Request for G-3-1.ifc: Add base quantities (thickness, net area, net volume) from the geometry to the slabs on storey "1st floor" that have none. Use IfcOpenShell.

First a look at what the model holds.

```python
import ifcopenshell
import ifcopenshell.util.element
import ifcopenshell.util.unit

model = ifcopenshell.open("G-3-1.ifc")
print(model.schema)
for unit_type in ("LENGTHUNIT", "AREAUNIT", "VOLUMEUNIT"):
    print(unit_type, ifcopenshell.util.unit.calculate_unit_scale(model, unit_type))
storey = next(s for s in model.by_type("IfcBuildingStorey") if s.Name == "1st floor")
slabs = [e for e in ifcopenshell.util.element.get_decomposition(storey) if e.is_a("IfcSlab")]
for e in sorted(slabs, key=lambda e: e.id()):
    print(e.id(), e.is_a(), e.Name, list(ifcopenshell.util.element.get_psets(e, qtos_only=True)), sep=" | ")
```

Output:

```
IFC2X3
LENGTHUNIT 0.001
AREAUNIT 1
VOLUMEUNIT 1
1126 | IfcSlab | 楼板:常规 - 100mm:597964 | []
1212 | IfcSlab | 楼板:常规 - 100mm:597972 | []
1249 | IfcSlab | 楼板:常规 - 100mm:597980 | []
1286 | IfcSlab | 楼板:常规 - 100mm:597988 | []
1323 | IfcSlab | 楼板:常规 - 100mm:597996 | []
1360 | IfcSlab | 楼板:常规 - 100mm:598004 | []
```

```python
import ifcopenshell
import ifcopenshell.api.pset
import ifcopenshell.geom
import ifcopenshell.util.element
import ifcopenshell.util.shape
import ifcopenshell.util.unit

model = ifcopenshell.open("G-3-1.ifc")
unit_scale = ifcopenshell.util.unit.calculate_unit_scale(model)
area_scale = ifcopenshell.util.unit.calculate_unit_scale(model, "AREAUNIT")
volume_scale = ifcopenshell.util.unit.calculate_unit_scale(model, "VOLUMEUNIT")
settings = ifcopenshell.geom.settings()

storey = next(s for s in model.by_type("IfcBuildingStorey") if s.Name == "1st floor")
slabs = [e for e in ifcopenshell.util.element.get_decomposition(storey) if e.is_a("IfcSlab")]

for e in sorted(slabs, key=lambda e: e.id()):
    if ifcopenshell.util.element.get_psets(e, qtos_only=True, should_inherit=False):
        continue
    # Geometry comes back in metres, in the element's own axes.
    shape = ifcopenshell.geom.create_shape(settings, e)
    values = {
        "Width": ifcopenshell.util.shape.get_z(shape.geometry) / unit_scale,
        "NetArea": ifcopenshell.util.shape.get_footprint_area(shape.geometry) / area_scale,
        "NetVolume": ifcopenshell.util.shape.get_volume(shape.geometry) / volume_scale,
    }
    qto = ifcopenshell.api.pset.add_qto(model, product=e, name="BaseQuantities")
    ifcopenshell.api.pset.edit_qto(model, qto=qto, properties=values)
    print(e.id(), {k: round(v, 3) for k, v in values.items()})

model.write("G-3-1-out.ifc")
```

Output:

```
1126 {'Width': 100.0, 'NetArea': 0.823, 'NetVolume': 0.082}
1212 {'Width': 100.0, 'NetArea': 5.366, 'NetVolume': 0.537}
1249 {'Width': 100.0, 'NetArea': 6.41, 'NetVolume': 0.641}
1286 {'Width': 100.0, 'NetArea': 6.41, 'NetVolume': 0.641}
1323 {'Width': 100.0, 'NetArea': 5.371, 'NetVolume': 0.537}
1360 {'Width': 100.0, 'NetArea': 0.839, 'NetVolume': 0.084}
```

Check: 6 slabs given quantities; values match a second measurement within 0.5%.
